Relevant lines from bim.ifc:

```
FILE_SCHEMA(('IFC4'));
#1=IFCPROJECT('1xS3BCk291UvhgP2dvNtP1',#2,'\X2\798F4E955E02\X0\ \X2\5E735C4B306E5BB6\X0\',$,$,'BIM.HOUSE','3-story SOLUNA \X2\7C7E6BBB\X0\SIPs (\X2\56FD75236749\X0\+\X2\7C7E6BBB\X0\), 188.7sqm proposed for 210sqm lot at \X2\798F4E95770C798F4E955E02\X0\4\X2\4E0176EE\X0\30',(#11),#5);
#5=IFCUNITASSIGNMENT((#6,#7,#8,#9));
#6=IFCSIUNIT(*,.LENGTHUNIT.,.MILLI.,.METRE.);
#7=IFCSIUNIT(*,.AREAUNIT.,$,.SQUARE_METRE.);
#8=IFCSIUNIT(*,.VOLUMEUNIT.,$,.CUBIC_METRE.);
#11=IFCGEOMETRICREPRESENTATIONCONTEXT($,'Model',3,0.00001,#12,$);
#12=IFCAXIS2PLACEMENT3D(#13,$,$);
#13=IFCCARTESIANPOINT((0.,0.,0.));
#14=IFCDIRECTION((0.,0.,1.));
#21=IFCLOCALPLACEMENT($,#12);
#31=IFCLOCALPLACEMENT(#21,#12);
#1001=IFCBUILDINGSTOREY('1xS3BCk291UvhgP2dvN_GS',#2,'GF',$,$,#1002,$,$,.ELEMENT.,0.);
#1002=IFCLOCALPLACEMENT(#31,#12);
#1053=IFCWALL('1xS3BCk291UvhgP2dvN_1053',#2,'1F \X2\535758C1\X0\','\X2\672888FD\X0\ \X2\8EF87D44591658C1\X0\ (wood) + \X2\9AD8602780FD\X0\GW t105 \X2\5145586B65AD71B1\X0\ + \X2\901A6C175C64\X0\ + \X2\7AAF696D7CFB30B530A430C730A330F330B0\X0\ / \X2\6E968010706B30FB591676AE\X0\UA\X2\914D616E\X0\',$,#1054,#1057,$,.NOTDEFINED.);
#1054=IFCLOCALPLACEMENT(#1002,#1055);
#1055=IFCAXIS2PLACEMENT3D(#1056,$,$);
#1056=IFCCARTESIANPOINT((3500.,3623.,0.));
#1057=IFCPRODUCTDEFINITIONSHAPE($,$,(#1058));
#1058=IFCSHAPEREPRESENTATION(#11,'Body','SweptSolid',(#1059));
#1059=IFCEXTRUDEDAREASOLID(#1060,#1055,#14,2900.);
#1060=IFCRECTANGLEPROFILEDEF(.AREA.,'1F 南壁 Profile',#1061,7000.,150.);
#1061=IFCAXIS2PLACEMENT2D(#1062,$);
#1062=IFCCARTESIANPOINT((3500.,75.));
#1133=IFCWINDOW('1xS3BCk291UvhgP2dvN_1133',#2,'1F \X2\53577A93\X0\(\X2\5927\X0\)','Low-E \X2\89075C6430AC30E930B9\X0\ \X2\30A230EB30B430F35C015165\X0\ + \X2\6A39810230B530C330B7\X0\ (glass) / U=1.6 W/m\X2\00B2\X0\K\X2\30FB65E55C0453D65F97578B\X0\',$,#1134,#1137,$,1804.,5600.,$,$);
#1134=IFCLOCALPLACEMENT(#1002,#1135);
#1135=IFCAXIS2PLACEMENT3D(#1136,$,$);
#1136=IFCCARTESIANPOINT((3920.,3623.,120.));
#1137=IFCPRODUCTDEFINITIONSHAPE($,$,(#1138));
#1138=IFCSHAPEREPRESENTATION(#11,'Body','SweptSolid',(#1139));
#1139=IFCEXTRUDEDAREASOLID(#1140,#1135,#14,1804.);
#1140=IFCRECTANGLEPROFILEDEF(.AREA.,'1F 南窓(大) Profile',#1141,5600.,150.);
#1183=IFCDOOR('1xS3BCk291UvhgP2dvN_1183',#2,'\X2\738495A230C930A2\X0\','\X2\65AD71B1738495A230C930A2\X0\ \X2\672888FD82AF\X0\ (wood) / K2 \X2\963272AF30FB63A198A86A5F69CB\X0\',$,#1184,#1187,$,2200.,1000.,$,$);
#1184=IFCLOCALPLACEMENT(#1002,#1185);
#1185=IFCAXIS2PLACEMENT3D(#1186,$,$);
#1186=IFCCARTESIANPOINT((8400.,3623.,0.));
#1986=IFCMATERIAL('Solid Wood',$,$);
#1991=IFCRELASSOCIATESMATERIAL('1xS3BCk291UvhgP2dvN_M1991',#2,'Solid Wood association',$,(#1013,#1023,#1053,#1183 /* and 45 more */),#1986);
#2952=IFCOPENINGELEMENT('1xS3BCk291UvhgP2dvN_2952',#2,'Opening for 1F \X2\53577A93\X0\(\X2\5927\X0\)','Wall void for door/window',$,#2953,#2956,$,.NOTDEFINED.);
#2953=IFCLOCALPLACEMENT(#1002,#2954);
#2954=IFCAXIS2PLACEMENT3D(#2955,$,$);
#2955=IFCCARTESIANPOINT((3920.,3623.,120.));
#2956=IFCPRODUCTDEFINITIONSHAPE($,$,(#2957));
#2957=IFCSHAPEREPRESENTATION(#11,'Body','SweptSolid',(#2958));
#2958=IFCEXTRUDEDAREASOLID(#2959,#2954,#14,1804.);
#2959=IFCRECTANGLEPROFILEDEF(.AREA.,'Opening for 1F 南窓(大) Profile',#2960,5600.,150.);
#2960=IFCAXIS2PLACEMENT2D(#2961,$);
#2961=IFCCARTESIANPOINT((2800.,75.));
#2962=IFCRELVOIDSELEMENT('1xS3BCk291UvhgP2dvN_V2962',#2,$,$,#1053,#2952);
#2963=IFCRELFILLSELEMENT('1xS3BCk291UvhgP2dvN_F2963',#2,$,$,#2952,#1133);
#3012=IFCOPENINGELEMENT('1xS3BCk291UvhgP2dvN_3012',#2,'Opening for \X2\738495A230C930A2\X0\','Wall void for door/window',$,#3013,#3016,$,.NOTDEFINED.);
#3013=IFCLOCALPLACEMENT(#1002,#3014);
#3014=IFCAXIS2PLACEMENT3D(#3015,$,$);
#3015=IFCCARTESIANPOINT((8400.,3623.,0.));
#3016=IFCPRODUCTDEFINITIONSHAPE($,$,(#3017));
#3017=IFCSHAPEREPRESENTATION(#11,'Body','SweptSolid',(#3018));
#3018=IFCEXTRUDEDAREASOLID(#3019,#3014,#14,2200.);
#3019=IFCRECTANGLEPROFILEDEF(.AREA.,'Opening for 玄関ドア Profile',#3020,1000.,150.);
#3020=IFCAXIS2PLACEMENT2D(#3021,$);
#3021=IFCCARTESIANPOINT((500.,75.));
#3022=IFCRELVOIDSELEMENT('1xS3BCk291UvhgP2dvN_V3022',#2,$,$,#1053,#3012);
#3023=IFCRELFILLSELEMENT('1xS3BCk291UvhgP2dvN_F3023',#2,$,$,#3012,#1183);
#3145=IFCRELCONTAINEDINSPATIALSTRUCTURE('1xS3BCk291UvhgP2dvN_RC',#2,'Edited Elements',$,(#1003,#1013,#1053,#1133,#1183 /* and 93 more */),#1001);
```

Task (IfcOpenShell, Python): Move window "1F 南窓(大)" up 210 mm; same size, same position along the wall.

```python
import numpy as np
import ifcopenshell
import ifcopenshell.api.geometry
import ifcopenshell.util.placement
import ifcopenshell.util.unit

model = ifcopenshell.open("bim.ifc")
unit_scale = ifcopenshell.util.unit.calculate_unit_scale(model)

window = model.by_guid("1xS3BCk291UvhgP2dvN_1133")
opening = window.FillsVoids[0].RelatingOpeningElement
dz = 0.21 / unit_scale

shift = np.array([0.0, 0.0, dz])
# The window is not placed relative to its opening, so move both.
for product in (opening, window):
    matrix = ifcopenshell.util.placement.get_local_placement(product.ObjectPlacement)
    matrix[:3, 3] += shift
    ifcopenshell.api.geometry.edit_object_placement(model, product=product, matrix=matrix, is_si=False)

print(f"moved by {dz * unit_scale:+.3f} m")

model.write("bim_updated.ifc")
```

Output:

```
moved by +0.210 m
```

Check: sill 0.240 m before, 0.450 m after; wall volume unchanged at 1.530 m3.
